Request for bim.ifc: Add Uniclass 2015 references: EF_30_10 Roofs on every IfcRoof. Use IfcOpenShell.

First a look at what the model holds.

```python
import ifcopenshell

model = ifcopenshell.open("bim.ifc")
print(model.schema)
print("classifications:", [c.Name for c in model.by_type("IfcClassification")])
for ifc_class in ("IfcDoor", "IfcRoof", "IfcStair", "IfcWall", "IfcWindow"):
    print(ifc_class, len(model.by_type(ifc_class)))
```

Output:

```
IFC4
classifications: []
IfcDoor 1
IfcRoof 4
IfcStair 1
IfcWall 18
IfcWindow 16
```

```python
import ifcopenshell
import ifcopenshell.api.classification

model = ifcopenshell.open("bim.ifc")

system = ifcopenshell.api.classification.add_classification(model, classification="Uniclass 2015")

codes = {
    "IfcRoof": ("EF_30_10", "Roofs"),
}
for ifc_class, (code, name) in codes.items():
    products = model.by_type(ifc_class)
    ifcopenshell.api.classification.add_reference(
        model, products=products, classification=system, identification=code, name=name
    )
    print(code, len(products))

model.write("bim_v2.ifc")
```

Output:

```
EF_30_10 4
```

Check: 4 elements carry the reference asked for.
